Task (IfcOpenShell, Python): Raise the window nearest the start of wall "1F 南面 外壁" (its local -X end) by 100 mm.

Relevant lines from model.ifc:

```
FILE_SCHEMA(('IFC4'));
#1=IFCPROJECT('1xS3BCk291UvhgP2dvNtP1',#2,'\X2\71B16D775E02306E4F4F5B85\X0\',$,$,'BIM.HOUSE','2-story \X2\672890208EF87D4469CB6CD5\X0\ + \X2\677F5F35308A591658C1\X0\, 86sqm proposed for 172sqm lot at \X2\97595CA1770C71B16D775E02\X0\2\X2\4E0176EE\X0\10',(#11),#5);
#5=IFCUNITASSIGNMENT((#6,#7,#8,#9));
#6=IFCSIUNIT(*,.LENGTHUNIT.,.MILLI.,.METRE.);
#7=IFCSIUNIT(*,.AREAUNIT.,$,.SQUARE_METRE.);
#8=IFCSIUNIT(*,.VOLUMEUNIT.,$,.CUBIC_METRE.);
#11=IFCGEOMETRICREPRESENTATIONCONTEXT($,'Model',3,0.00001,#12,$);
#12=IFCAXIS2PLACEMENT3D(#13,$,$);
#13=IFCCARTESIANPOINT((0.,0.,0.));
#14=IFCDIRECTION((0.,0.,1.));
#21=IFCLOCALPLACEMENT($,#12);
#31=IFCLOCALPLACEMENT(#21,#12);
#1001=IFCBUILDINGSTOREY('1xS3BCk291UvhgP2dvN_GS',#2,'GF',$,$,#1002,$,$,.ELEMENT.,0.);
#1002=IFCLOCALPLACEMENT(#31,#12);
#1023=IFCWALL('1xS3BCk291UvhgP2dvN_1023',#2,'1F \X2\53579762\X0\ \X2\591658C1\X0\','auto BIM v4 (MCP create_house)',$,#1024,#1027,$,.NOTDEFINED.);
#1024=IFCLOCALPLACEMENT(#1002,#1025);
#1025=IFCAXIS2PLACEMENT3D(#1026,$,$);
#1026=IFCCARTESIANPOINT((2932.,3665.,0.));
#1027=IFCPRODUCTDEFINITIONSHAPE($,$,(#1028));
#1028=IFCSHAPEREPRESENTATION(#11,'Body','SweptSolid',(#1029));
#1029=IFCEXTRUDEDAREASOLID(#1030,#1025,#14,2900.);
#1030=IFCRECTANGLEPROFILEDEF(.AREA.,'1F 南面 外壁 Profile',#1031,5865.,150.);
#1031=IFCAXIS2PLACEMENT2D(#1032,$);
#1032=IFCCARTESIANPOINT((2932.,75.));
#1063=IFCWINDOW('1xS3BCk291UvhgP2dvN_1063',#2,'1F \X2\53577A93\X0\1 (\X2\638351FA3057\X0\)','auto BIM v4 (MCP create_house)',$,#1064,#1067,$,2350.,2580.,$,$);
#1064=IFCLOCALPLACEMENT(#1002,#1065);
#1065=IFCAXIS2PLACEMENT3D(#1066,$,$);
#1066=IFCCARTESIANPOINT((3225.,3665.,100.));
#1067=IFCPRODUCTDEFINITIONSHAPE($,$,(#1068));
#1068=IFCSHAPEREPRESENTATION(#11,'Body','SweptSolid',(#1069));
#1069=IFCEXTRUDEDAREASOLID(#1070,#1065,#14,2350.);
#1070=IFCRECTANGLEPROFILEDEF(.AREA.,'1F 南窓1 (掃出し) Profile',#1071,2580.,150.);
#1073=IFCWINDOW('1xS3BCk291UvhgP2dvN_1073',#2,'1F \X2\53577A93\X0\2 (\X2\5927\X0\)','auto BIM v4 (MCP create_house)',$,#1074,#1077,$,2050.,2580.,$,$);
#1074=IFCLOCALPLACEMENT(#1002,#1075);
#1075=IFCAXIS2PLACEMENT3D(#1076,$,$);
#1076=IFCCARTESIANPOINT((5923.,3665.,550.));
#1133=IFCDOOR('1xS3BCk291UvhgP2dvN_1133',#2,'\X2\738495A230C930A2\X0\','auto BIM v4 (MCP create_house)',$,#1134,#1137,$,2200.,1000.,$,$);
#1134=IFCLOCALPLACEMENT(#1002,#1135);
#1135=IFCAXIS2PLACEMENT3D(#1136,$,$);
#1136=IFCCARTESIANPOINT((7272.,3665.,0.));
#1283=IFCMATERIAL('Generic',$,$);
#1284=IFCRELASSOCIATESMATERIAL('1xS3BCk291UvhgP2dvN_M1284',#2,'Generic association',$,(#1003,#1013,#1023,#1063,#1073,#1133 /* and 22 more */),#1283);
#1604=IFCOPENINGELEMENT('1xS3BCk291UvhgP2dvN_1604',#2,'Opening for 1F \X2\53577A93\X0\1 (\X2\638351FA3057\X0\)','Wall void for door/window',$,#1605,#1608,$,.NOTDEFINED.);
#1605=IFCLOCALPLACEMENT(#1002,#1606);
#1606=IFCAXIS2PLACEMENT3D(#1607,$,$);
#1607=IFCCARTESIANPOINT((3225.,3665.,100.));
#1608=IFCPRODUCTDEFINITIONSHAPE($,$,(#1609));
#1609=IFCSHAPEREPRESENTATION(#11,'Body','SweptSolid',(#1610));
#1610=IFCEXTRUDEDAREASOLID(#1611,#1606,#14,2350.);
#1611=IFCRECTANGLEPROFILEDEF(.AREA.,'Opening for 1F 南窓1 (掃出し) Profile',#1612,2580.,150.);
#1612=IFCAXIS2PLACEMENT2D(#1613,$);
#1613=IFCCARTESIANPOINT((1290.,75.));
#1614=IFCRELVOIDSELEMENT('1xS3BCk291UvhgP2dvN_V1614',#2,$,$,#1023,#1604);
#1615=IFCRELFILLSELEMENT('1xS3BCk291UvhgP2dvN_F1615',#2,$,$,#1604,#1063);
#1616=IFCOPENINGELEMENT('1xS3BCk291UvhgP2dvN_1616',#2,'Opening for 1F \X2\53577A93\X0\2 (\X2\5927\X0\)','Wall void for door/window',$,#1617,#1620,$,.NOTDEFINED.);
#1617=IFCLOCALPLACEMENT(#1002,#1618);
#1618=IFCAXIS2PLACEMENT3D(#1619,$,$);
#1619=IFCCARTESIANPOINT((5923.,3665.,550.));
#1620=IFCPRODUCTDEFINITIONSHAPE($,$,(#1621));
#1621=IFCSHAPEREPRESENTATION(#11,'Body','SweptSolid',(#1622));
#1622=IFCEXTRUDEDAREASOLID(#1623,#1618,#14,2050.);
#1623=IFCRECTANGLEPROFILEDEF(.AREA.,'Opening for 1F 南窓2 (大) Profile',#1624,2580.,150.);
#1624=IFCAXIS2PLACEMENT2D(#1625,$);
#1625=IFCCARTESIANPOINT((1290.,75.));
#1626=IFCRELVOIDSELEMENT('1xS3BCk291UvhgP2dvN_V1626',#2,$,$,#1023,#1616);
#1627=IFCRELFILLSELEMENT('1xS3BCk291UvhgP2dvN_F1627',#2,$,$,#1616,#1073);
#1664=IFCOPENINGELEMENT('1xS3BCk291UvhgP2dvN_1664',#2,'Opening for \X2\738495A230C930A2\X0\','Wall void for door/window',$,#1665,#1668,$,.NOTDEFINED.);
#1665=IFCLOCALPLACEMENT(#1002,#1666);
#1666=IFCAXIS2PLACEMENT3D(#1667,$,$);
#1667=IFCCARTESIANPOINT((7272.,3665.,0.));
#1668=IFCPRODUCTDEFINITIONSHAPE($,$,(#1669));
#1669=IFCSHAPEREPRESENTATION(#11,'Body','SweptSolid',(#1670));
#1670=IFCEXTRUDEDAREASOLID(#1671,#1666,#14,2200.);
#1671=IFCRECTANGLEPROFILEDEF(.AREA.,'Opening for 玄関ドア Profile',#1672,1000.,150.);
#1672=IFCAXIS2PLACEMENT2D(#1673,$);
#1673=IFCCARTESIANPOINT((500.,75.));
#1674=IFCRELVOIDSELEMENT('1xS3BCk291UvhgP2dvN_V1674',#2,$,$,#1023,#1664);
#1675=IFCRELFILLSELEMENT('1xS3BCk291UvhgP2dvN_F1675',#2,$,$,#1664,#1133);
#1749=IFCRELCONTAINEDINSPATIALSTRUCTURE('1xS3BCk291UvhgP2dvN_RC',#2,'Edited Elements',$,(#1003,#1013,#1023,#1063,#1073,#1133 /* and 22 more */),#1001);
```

```python
import numpy as np
import ifcopenshell
import ifcopenshell.api.geometry
import ifcopenshell.util.placement
import ifcopenshell.util.unit

model = ifcopenshell.open("model.ifc")
unit_scale = ifcopenshell.util.unit.calculate_unit_scale(model)

window = model.by_guid("1xS3BCk291UvhgP2dvN_1063")
opening = window.FillsVoids[0].RelatingOpeningElement
dz = 100.0

shift = np.array([0.0, 0.0, dz])
# The window is not placed relative to its opening, so move both.
for product in (opening, window):
    matrix = ifcopenshell.util.placement.get_local_placement(product.ObjectPlacement)
    matrix[:3, 3] += shift
    ifcopenshell.api.geometry.edit_object_placement(model, product=product, matrix=matrix, is_si=False)

print(f"moved by {dz * unit_scale:+.3f} m")

model.write("model_edited.ifc")
```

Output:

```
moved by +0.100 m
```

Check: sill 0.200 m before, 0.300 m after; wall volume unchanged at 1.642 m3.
